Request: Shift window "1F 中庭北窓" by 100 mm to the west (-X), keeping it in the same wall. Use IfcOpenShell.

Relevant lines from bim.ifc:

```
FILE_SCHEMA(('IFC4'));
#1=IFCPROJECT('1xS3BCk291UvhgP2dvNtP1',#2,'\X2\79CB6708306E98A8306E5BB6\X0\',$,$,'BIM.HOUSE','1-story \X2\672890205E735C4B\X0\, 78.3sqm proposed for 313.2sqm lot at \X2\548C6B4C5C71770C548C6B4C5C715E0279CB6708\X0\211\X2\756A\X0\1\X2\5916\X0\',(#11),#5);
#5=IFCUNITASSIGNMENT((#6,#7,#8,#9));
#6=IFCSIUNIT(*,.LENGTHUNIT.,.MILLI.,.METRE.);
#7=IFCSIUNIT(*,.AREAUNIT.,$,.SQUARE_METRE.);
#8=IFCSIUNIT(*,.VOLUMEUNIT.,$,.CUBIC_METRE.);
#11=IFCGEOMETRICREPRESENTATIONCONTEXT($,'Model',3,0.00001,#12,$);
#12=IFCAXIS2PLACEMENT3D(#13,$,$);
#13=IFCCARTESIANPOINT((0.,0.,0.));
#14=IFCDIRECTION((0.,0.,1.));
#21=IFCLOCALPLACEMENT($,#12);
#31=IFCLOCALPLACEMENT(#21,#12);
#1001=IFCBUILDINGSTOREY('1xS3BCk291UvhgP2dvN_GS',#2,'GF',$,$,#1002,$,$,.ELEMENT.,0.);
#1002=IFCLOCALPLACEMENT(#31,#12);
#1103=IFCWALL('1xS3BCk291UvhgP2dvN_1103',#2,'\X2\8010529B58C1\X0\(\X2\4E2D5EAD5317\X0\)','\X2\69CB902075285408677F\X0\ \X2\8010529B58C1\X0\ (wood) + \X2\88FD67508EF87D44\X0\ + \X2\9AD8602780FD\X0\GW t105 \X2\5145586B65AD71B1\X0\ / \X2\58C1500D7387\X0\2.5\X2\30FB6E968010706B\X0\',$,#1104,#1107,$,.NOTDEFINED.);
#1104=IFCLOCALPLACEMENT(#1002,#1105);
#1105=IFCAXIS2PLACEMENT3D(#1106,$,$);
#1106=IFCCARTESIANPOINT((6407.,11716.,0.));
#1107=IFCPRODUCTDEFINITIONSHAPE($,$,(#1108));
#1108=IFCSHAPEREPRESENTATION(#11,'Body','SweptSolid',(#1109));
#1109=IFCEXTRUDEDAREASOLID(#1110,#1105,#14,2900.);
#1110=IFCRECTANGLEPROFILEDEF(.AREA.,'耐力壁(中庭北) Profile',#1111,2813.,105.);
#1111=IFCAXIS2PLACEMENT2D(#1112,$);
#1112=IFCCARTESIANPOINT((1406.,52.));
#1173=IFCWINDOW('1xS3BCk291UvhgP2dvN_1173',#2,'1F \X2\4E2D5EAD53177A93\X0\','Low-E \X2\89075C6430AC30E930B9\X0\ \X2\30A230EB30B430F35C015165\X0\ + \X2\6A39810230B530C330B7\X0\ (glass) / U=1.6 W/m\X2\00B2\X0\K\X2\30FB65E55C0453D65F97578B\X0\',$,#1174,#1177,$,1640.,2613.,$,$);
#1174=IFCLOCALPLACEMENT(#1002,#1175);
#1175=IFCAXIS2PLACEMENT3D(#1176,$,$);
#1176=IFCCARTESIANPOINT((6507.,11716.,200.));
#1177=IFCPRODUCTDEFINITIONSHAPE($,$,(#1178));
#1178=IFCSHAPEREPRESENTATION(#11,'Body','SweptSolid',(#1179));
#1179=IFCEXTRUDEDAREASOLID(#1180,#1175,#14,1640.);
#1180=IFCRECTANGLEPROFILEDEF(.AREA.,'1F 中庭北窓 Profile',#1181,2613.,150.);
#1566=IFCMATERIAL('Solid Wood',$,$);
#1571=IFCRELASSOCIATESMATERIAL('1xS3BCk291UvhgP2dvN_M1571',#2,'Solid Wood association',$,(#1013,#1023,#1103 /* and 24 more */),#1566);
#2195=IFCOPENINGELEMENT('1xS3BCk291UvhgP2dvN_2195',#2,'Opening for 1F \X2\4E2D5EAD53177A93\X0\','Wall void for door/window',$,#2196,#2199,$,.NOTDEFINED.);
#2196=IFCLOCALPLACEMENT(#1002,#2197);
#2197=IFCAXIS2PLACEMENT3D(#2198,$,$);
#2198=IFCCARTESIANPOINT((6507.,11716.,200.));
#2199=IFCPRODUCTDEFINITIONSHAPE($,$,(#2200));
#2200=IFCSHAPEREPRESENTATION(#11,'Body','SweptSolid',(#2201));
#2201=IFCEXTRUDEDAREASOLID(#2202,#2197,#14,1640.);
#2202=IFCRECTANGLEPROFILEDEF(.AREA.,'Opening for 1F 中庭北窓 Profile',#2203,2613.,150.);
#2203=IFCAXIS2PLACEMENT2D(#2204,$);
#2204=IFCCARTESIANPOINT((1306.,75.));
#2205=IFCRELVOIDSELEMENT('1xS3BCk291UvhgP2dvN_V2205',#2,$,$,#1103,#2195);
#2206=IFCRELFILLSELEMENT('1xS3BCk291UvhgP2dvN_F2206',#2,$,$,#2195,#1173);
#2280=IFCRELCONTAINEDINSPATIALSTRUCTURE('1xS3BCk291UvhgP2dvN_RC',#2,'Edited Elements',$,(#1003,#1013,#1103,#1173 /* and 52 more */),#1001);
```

```python
import ifcopenshell
import ifcopenshell.api.geometry
import ifcopenshell.util.placement
import ifcopenshell.util.unit

model = ifcopenshell.open("bim.ifc")
unit_scale = ifcopenshell.util.unit.calculate_unit_scale(model)

window = model.by_id(1173)
opening = window.FillsVoids[0].RelatingOpeningElement
wall = opening.VoidsElements[0].RelatingBuildingElement

wall_matrix = ifcopenshell.util.placement.get_local_placement(wall.ObjectPlacement)
shift = wall_matrix[:3, 0] * -0.1 / unit_scale
before = ifcopenshell.util.placement.get_local_placement(window.ObjectPlacement)[:3, 3].copy()

# The window is not placed relative to its opening, so move both.
for product in (opening, window):
    matrix = ifcopenshell.util.placement.get_local_placement(product.ObjectPlacement)
    matrix[:3, 3] += shift
    ifcopenshell.api.geometry.edit_object_placement(model, product=product, matrix=matrix, is_si=False)

after = ifcopenshell.util.placement.get_local_placement(window.ObjectPlacement)[:3, 3]
print("window moved by", (after - before).round(3) + 0.0)

model.write("bim-out.ifc")
```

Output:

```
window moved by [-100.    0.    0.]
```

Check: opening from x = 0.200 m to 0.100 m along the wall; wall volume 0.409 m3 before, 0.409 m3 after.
